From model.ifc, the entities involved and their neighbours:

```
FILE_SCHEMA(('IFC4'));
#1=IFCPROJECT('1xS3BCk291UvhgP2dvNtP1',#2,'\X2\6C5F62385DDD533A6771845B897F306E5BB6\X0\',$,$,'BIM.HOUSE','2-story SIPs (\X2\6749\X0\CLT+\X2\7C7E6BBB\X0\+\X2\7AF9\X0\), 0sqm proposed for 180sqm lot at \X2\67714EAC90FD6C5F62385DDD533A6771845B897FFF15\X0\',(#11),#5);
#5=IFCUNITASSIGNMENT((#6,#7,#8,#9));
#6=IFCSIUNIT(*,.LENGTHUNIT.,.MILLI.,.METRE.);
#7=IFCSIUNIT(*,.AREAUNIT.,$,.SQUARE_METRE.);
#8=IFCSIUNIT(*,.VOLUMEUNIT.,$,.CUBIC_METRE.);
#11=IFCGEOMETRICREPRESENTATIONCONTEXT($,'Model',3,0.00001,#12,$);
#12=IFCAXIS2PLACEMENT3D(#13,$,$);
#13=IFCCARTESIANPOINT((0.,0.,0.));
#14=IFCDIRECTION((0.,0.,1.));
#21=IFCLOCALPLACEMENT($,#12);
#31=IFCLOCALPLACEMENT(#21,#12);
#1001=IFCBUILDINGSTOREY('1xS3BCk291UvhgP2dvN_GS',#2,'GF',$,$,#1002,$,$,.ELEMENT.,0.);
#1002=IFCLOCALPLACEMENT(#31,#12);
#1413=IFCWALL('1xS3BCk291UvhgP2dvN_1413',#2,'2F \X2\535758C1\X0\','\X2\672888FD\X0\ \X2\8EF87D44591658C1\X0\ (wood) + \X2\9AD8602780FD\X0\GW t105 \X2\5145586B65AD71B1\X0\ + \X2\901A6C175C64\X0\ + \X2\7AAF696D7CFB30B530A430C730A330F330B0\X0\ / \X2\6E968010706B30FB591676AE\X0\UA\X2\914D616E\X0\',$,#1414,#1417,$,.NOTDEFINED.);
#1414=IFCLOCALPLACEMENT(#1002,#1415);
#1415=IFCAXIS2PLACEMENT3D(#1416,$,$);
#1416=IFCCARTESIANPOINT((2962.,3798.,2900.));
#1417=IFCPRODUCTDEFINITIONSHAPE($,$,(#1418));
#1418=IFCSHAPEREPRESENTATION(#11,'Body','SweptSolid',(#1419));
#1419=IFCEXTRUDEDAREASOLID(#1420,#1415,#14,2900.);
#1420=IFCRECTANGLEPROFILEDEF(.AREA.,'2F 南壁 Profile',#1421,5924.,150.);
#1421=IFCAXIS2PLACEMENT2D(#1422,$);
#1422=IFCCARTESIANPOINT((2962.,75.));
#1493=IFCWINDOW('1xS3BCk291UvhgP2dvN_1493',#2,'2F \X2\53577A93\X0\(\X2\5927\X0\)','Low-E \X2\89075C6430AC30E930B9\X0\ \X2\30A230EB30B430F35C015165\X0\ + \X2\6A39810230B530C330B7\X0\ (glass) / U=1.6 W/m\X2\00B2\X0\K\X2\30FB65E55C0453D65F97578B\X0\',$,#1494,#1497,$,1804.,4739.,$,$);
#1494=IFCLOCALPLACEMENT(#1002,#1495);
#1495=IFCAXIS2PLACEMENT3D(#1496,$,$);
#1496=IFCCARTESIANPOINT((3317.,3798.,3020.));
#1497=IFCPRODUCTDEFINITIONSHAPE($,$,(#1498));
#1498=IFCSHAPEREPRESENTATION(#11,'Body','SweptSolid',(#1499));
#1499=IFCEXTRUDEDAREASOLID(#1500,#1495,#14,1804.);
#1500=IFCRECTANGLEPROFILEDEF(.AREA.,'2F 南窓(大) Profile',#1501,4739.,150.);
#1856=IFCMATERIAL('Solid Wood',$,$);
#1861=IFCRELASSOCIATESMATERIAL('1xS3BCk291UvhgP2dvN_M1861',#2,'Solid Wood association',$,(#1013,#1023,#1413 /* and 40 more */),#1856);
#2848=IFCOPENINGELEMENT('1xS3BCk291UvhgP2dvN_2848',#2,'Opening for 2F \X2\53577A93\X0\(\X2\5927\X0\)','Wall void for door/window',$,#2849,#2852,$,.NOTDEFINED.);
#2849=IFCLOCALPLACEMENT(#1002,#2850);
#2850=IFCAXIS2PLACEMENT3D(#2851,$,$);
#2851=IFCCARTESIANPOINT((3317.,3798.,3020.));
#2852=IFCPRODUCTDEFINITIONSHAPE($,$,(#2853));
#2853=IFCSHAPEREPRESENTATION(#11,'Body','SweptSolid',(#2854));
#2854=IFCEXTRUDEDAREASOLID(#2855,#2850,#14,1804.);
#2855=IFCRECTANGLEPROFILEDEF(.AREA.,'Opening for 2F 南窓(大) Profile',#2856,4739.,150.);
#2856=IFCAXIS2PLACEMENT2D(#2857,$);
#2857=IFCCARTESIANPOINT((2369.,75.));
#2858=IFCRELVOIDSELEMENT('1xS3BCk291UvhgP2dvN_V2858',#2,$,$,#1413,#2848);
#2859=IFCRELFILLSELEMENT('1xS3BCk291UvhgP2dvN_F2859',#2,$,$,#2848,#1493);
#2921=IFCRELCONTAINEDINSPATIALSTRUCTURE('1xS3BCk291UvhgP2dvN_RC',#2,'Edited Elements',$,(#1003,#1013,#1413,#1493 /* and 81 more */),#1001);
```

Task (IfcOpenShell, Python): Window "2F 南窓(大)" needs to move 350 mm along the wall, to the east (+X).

```python
import ifcopenshell
import ifcopenshell.api.geometry
import ifcopenshell.util.placement

model = ifcopenshell.open("model.ifc")

window = model.by_guid("1xS3BCk291UvhgP2dvN_1493")
opening = window.FillsVoids[0].RelatingOpeningElement
wall = opening.VoidsElements[0].RelatingBuildingElement

wall_matrix = ifcopenshell.util.placement.get_local_placement(wall.ObjectPlacement)
shift = wall_matrix[:3, 0] * 350.0
before = ifcopenshell.util.placement.get_local_placement(window.ObjectPlacement)[:3, 3].copy()

# The window is not placed relative to its opening, so move both.
for product in (opening, window):
    matrix = ifcopenshell.util.placement.get_local_placement(product.ObjectPlacement)
    matrix[:3, 3] += shift
    ifcopenshell.api.geometry.edit_object_placement(model, product=product, matrix=matrix, is_si=False)

after = ifcopenshell.util.placement.get_local_placement(window.ObjectPlacement)[:3, 3]
print("window moved by", (after - before).round(3) + 0.0)

model.write("model_rev.ifc")
```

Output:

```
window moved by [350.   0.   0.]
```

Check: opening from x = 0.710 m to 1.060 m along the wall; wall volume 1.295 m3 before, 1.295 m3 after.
